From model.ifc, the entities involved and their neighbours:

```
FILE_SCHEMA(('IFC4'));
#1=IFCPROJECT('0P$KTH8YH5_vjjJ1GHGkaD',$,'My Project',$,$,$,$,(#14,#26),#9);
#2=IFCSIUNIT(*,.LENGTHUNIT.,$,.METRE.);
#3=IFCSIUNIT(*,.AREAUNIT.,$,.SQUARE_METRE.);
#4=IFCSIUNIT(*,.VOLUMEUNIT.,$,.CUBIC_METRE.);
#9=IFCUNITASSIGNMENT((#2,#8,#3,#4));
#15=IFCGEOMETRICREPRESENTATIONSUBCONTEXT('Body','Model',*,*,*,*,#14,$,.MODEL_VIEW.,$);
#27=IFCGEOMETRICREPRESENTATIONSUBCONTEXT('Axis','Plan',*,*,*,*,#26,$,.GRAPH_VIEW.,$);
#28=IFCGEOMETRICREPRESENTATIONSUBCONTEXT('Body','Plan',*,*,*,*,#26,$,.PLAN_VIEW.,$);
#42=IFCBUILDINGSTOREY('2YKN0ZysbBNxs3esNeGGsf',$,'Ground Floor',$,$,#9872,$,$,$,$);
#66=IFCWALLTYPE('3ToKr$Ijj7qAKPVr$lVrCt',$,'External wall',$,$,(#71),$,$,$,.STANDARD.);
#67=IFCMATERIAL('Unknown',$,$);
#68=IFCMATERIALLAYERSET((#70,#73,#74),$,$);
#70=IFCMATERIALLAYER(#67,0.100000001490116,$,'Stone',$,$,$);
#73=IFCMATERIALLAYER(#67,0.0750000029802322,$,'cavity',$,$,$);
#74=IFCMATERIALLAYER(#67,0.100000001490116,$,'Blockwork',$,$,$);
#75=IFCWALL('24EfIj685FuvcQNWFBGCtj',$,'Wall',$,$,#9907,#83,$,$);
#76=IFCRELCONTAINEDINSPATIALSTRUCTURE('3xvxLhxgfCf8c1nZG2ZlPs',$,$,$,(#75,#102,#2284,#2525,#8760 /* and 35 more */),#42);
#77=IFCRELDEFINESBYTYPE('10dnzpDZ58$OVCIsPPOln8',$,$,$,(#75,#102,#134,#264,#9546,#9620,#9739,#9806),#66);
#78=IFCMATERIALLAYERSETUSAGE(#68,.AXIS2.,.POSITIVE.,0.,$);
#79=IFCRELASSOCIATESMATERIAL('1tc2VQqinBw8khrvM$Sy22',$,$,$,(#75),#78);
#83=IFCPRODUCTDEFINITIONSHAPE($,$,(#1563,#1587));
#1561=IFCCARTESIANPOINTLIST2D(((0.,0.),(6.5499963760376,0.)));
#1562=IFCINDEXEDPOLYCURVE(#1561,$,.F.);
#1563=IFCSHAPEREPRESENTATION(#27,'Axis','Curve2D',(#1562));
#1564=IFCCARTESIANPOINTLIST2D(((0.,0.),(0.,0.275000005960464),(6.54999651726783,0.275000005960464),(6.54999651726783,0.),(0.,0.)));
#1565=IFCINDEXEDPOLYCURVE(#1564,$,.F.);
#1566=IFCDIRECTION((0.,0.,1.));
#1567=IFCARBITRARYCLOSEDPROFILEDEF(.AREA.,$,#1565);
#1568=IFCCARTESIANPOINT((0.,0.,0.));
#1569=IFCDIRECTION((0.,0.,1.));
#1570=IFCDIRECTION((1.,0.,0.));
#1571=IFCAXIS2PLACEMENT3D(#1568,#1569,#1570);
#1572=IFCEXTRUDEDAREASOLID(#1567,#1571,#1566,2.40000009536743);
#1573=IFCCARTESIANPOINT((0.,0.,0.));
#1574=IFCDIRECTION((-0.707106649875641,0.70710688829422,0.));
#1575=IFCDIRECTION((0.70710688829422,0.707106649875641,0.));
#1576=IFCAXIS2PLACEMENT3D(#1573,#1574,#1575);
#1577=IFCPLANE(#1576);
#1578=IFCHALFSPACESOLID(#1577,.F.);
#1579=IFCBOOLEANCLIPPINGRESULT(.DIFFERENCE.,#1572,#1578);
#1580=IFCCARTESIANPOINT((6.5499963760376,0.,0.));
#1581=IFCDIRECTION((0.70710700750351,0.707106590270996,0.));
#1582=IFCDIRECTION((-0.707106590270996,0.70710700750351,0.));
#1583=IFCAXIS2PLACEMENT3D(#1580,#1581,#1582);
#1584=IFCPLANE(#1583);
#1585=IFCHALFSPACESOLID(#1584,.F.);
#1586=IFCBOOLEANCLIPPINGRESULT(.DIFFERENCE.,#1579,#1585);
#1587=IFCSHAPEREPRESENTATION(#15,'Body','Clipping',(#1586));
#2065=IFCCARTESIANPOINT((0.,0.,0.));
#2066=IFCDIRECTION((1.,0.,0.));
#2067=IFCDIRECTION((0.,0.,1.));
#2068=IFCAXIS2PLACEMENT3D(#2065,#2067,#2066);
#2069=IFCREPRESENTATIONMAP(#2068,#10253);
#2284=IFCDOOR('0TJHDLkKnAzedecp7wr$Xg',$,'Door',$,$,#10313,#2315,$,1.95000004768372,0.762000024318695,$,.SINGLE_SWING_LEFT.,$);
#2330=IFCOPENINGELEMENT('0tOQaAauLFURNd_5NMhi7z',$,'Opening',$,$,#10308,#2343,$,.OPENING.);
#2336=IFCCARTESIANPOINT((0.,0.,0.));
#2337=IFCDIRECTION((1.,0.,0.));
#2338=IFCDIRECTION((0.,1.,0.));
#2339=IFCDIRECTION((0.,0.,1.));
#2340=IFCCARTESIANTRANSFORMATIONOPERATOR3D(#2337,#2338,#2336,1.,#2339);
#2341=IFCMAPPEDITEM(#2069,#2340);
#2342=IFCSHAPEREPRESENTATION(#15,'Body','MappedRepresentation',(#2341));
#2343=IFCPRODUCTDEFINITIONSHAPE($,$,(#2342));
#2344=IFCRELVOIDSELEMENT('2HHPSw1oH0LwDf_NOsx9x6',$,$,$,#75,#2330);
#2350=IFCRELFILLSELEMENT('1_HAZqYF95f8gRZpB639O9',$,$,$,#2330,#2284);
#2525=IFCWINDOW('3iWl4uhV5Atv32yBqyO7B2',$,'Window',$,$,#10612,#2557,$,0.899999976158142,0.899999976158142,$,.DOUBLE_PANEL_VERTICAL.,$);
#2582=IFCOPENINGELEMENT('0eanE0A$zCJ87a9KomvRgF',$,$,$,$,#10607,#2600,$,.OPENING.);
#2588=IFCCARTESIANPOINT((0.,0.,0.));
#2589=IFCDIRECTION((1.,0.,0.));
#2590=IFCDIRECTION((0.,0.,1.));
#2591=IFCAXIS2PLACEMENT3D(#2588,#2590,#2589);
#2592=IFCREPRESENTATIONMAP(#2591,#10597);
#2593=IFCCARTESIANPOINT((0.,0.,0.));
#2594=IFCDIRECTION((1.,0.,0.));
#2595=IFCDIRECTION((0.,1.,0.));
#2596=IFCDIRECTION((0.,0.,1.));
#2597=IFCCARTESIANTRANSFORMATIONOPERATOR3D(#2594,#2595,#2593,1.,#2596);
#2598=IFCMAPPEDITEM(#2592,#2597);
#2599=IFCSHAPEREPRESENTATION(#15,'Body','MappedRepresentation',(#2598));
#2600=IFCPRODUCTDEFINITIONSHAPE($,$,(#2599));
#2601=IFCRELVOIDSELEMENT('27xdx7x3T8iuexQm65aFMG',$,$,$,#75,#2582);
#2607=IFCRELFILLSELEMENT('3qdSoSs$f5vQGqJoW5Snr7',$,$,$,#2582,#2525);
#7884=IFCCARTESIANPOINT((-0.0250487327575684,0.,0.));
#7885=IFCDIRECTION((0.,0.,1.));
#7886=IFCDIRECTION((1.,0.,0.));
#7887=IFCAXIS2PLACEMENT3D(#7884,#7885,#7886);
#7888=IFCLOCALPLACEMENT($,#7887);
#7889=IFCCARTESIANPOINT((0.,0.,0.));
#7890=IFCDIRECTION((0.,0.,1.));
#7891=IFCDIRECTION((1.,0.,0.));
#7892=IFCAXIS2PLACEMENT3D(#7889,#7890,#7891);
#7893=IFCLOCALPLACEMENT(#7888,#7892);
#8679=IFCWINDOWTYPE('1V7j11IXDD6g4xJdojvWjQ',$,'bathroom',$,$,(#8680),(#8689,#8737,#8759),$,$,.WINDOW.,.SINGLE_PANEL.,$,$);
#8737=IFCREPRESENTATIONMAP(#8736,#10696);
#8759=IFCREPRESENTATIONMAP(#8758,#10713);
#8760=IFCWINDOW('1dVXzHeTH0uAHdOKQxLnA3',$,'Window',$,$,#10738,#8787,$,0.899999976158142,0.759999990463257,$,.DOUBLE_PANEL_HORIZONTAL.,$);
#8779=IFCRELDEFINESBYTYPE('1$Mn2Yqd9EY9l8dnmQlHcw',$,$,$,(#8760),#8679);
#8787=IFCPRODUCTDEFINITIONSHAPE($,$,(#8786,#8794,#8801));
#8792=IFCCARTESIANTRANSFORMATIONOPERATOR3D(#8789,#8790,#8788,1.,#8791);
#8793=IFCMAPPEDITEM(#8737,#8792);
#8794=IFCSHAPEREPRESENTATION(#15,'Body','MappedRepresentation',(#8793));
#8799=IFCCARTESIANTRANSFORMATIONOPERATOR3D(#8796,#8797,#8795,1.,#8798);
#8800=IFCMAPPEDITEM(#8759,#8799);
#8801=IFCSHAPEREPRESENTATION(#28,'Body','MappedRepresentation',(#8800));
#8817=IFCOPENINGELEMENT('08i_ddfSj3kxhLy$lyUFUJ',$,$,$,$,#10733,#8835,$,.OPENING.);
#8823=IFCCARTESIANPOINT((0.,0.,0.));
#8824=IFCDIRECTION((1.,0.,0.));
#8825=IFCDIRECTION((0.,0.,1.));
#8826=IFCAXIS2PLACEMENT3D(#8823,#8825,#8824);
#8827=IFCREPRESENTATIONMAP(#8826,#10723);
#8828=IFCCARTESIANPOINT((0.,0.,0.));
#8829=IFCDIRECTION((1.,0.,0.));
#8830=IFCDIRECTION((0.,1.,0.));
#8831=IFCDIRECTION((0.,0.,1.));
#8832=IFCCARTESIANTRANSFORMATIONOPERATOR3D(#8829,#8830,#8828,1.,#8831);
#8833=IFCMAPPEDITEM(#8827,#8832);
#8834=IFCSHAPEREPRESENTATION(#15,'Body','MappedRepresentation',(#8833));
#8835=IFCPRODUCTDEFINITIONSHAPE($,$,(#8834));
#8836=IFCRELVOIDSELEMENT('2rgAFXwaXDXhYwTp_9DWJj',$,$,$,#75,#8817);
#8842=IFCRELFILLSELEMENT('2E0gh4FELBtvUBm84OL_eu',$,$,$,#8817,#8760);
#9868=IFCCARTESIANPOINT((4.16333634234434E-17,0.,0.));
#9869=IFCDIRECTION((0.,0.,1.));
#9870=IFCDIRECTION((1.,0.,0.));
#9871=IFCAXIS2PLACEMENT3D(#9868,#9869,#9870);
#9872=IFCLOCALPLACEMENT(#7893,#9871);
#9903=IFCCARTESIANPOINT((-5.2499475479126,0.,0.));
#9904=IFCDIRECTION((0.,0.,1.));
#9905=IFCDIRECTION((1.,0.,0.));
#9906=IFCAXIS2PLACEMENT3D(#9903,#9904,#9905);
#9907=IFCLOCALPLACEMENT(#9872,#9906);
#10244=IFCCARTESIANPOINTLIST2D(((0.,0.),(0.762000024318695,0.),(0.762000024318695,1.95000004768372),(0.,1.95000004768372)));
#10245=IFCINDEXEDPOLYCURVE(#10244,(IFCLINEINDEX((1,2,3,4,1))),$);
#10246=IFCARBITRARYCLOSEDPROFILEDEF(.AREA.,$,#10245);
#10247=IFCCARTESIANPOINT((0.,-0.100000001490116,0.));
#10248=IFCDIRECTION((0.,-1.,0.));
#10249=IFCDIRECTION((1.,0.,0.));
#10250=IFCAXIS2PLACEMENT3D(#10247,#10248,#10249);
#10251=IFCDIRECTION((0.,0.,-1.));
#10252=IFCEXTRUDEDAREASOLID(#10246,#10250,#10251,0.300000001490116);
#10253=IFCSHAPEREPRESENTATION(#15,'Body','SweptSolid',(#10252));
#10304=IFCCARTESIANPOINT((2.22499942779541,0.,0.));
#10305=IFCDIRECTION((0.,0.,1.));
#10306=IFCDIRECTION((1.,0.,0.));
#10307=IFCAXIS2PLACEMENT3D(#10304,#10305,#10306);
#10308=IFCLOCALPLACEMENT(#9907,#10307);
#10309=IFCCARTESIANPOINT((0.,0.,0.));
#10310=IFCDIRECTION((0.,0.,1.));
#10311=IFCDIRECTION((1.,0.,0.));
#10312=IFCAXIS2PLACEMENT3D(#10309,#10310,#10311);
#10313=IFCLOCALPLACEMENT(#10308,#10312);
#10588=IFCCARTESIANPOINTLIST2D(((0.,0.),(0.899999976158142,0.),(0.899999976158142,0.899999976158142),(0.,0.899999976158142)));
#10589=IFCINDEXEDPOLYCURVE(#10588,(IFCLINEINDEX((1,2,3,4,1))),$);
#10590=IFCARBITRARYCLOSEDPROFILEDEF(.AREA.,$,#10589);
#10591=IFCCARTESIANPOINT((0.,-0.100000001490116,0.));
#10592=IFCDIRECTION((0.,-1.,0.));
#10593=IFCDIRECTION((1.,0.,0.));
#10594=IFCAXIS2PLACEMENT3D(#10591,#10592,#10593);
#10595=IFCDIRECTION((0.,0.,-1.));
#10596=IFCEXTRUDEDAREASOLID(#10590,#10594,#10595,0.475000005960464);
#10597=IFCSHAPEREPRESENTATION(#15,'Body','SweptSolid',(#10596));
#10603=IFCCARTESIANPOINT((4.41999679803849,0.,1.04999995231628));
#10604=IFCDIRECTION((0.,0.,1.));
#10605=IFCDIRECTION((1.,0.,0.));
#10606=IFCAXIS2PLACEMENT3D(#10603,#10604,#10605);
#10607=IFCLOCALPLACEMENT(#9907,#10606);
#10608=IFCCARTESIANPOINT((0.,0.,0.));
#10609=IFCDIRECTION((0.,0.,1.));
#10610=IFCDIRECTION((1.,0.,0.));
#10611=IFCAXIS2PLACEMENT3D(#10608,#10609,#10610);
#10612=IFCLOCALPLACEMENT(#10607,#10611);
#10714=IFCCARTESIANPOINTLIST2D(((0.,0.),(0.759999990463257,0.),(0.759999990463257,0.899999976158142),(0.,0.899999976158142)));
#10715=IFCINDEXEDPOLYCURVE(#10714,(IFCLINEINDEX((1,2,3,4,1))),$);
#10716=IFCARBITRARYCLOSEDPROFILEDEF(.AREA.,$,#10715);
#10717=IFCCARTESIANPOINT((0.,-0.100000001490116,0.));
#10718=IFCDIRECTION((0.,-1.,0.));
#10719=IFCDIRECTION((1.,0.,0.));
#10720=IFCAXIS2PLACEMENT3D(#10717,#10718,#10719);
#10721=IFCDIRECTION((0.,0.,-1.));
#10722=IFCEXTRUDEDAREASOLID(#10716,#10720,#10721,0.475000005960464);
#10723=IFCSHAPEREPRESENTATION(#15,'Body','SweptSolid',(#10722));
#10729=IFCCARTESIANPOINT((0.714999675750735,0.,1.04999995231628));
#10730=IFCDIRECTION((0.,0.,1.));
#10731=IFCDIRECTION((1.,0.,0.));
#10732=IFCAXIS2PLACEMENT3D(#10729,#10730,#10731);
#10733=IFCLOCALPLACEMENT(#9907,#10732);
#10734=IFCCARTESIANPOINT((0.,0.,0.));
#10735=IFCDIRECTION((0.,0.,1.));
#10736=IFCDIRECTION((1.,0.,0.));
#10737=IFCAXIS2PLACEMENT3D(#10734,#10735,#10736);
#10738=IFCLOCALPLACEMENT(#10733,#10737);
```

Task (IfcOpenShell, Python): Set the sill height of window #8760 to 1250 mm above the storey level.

```python
import numpy as np
import ifcopenshell
import ifcopenshell.api.geometry
import ifcopenshell.geom
import ifcopenshell.util.element
import ifcopenshell.util.placement
import ifcopenshell.util.shape
import ifcopenshell.util.unit

model = ifcopenshell.open("model.ifc")
unit_scale = ifcopenshell.util.unit.calculate_unit_scale(model)

window = model.by_guid("1dVXzHeTH0uAHdOKQxLnA3")
opening = window.FillsVoids[0].RelatingOpeningElement
storey = ifcopenshell.util.element.get_container(window, ifc_class="IfcBuildingStorey")
level = ifcopenshell.util.placement.get_local_placement(storey.ObjectPlacement)[2, 3]

# The opening's origin need not be at the sill, so measure its lowest point.
shape = ifcopenshell.geom.create_shape(ifcopenshell.geom.settings(), opening)
bottom = ifcopenshell.util.shape.get_shape_bottom_elevation(shape, shape.geometry) / unit_scale
dz = level + 1.25 - bottom

shift = np.array([0.0, 0.0, dz])
# The window is placed relative to its opening, so it follows when the opening moves.
matrix = ifcopenshell.util.placement.get_local_placement(opening.ObjectPlacement)
matrix[:3, 3] += shift
ifcopenshell.api.geometry.edit_object_placement(
    model, product=opening, matrix=matrix, is_si=False, should_transform_children=True
)

print(f"moved by {dz * unit_scale:+.3f} m")

model.write("model_rev.ifc")
```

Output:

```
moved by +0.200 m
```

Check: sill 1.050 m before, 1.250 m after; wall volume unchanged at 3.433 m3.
